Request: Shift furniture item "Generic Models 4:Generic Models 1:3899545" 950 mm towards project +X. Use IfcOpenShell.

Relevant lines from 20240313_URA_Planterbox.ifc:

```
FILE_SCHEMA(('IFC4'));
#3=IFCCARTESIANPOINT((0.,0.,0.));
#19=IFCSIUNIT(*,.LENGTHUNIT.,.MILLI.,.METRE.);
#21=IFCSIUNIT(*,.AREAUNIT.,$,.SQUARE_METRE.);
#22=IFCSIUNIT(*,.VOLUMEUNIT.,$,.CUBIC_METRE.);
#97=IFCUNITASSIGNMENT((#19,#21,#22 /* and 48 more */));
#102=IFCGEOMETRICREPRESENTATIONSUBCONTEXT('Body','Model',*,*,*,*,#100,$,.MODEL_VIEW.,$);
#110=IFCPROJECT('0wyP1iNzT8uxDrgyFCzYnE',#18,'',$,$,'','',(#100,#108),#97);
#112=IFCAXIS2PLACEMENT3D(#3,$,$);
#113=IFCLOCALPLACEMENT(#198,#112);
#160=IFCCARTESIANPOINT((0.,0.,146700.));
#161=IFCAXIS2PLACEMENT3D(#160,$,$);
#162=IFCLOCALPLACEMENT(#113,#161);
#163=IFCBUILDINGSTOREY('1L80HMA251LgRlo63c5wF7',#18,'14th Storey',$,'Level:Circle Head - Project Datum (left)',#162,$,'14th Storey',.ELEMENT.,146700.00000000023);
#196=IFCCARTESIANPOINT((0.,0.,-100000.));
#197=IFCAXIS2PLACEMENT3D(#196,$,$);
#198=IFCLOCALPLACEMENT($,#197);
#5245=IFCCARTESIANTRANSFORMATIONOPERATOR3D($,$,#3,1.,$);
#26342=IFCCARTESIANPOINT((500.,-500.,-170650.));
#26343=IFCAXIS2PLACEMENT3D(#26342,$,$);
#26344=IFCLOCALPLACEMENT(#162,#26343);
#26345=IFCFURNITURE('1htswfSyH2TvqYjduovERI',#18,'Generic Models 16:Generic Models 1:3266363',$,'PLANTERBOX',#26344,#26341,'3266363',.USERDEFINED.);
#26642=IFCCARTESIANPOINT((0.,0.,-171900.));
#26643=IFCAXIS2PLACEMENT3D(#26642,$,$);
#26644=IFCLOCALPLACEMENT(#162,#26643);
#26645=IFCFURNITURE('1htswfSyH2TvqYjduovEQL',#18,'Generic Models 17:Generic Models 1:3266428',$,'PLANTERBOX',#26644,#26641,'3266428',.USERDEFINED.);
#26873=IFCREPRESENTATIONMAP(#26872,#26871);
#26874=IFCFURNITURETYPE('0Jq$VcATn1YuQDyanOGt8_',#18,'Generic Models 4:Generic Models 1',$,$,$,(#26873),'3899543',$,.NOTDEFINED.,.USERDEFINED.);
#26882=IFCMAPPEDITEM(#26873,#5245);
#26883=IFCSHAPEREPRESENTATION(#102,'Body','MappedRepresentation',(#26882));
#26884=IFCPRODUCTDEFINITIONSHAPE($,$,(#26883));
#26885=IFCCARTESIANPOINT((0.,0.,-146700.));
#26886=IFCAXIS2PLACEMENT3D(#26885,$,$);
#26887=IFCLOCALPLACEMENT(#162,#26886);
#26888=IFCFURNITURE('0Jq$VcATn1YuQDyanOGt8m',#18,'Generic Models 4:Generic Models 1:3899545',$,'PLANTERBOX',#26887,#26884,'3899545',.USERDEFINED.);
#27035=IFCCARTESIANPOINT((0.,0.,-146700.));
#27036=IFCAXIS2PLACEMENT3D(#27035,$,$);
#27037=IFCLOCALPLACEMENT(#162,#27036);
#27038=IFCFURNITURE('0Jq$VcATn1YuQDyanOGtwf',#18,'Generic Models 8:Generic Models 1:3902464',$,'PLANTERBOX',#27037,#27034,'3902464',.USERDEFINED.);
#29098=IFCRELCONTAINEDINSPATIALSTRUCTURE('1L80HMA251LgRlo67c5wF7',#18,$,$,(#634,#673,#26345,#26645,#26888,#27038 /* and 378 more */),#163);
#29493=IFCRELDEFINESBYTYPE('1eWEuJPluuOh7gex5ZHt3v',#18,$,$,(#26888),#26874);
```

```python
import ifcopenshell
import ifcopenshell.api.geometry
import ifcopenshell.util.placement

model = ifcopenshell.open("20240313_URA_Planterbox.ifc")

item = model.by_guid("0Jq$VcATn1YuQDyanOGt8m")
matrix = ifcopenshell.util.placement.get_local_placement(item.ObjectPlacement)
matrix[0, 3] += 950.0
ifcopenshell.api.geometry.edit_object_placement(model, product=item, matrix=matrix, is_si=False)

print(ifcopenshell.util.placement.get_local_placement(item.ObjectPlacement).round(3) + 0.0)

model.write("20240313_URA_Planterbox_updated.ifc")
```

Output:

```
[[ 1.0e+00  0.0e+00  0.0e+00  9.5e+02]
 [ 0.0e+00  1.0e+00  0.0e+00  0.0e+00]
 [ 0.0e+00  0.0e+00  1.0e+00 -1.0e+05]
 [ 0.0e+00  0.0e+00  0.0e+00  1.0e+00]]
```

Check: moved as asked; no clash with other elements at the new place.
